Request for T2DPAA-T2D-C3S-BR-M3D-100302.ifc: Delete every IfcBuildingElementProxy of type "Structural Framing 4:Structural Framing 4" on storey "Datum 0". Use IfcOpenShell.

First a look at what the model holds.

```python
import ifcopenshell
import ifcopenshell.util.element

model = ifcopenshell.open("T2DPAA-T2D-C3S-BR-M3D-100302.ifc")
print(model.schema)
storey = next(s for s in model.by_type("IfcBuildingStorey") if s.Name == "Datum 0")
proxies = [e for e in ifcopenshell.util.element.get_decomposition(storey) if e.is_a("IfcBuildingElementProxy")]
seen = {}
for e in proxies:
    element_type = ifcopenshell.util.element.get_type(e)
    name = element_type.Name if element_type not in (None, e) else None
    seen[name] = seen.get(name, 0) + 1
for name, count in sorted(seen.items(), key=str):
    print(count, "x", name)
```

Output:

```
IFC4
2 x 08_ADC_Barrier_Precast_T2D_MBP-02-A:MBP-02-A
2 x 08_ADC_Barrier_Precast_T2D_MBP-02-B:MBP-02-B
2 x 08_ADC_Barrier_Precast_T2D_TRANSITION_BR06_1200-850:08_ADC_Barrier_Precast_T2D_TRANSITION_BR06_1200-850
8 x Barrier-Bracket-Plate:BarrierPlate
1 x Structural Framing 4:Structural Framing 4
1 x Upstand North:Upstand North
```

```python
import ifcopenshell
import ifcopenshell.api.root
import ifcopenshell.util.element

model = ifcopenshell.open("T2DPAA-T2D-C3S-BR-M3D-100302.ifc")

storey = next(s for s in model.by_type("IfcBuildingStorey") if s.Name == "Datum 0")
proxies = [e for e in ifcopenshell.util.element.get_decomposition(storey) if e.is_a("IfcBuildingElementProxy")]
targets = [e for e in proxies if (t := ifcopenshell.util.element.get_type(e)) not in (None, e) and t.Name == "Structural Framing 4:Structural Framing 4"]

for e in targets:
    ifcopenshell.api.root.remove_product(model, product=e)
print(len(targets), "removed")

model.write("T2DPAA-T2D-C3S-BR-M3D-100302_v2.ifc")
```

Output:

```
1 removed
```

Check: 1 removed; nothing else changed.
